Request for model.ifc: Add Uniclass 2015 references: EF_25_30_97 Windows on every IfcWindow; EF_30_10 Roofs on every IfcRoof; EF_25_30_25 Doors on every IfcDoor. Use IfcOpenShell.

First a look at what the model holds.

```python
import ifcopenshell

model = ifcopenshell.open("model.ifc")
print(model.schema)
print("classifications:", [c.Name for c in model.by_type("IfcClassification")])
for ifc_class in ("IfcDoor", "IfcRoof", "IfcStair", "IfcWall", "IfcWindow"):
    print(ifc_class, len(model.by_type(ifc_class)))
```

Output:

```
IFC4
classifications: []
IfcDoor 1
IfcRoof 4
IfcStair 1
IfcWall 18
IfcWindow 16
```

```python
import ifcopenshell
import ifcopenshell.api.classification

model = ifcopenshell.open("model.ifc")

system = ifcopenshell.api.classification.add_classification(model, classification="Uniclass 2015")

codes = {
    "IfcWindow": ("EF_25_30_97", "Windows"),
    "IfcRoof": ("EF_30_10", "Roofs"),
    "IfcDoor": ("EF_25_30_25", "Doors"),
}
for ifc_class, (code, name) in codes.items():
    products = model.by_type(ifc_class)
    ifcopenshell.api.classification.add_reference(
        model, products=products, classification=system, identification=code, name=name
    )
    print(code, len(products))

model.write("model_edited.ifc")
```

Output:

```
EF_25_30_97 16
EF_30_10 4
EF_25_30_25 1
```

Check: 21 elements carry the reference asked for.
